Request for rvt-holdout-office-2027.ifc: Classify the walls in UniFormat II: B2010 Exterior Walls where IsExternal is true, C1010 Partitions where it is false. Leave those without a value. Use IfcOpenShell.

First a look at what the model holds.

```python
import ifcopenshell
import ifcopenshell.util.element

model = ifcopenshell.open("rvt-holdout-office-2027.ifc")
print(model.schema)
print("classifications:", [c.Name for c in model.by_type("IfcClassification")])
values = [ifcopenshell.util.element.get_pset(e, "Pset_WallCommon", "IsExternal") for e in model.by_type("IfcWall")]
for value in (True, False, None):
    print("IsExternal", value, values.count(value))
```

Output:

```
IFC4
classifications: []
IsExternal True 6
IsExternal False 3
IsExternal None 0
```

```python
import ifcopenshell
import ifcopenshell.api.classification
import ifcopenshell.util.element

model = ifcopenshell.open("rvt-holdout-office-2027.ifc")

system = ifcopenshell.api.classification.add_classification(model, classification="UniFormat II")

walls = model.by_type("IfcWall")
external = {e: ifcopenshell.util.element.get_pset(e, "Pset_WallCommon", "IsExternal") for e in walls}
for flag, code, name in ((True, "B2010", "Exterior Walls"), (False, "C1010", "Partitions")):
    products = [e for e in walls if external[e] is flag]
    ifcopenshell.api.classification.add_reference(
        model, products=products, classification=system, identification=code, name=name
    )
    print(code, len(products))

model.write("rvt-holdout-office-2027_updated.ifc")
```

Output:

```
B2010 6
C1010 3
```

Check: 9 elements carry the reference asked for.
